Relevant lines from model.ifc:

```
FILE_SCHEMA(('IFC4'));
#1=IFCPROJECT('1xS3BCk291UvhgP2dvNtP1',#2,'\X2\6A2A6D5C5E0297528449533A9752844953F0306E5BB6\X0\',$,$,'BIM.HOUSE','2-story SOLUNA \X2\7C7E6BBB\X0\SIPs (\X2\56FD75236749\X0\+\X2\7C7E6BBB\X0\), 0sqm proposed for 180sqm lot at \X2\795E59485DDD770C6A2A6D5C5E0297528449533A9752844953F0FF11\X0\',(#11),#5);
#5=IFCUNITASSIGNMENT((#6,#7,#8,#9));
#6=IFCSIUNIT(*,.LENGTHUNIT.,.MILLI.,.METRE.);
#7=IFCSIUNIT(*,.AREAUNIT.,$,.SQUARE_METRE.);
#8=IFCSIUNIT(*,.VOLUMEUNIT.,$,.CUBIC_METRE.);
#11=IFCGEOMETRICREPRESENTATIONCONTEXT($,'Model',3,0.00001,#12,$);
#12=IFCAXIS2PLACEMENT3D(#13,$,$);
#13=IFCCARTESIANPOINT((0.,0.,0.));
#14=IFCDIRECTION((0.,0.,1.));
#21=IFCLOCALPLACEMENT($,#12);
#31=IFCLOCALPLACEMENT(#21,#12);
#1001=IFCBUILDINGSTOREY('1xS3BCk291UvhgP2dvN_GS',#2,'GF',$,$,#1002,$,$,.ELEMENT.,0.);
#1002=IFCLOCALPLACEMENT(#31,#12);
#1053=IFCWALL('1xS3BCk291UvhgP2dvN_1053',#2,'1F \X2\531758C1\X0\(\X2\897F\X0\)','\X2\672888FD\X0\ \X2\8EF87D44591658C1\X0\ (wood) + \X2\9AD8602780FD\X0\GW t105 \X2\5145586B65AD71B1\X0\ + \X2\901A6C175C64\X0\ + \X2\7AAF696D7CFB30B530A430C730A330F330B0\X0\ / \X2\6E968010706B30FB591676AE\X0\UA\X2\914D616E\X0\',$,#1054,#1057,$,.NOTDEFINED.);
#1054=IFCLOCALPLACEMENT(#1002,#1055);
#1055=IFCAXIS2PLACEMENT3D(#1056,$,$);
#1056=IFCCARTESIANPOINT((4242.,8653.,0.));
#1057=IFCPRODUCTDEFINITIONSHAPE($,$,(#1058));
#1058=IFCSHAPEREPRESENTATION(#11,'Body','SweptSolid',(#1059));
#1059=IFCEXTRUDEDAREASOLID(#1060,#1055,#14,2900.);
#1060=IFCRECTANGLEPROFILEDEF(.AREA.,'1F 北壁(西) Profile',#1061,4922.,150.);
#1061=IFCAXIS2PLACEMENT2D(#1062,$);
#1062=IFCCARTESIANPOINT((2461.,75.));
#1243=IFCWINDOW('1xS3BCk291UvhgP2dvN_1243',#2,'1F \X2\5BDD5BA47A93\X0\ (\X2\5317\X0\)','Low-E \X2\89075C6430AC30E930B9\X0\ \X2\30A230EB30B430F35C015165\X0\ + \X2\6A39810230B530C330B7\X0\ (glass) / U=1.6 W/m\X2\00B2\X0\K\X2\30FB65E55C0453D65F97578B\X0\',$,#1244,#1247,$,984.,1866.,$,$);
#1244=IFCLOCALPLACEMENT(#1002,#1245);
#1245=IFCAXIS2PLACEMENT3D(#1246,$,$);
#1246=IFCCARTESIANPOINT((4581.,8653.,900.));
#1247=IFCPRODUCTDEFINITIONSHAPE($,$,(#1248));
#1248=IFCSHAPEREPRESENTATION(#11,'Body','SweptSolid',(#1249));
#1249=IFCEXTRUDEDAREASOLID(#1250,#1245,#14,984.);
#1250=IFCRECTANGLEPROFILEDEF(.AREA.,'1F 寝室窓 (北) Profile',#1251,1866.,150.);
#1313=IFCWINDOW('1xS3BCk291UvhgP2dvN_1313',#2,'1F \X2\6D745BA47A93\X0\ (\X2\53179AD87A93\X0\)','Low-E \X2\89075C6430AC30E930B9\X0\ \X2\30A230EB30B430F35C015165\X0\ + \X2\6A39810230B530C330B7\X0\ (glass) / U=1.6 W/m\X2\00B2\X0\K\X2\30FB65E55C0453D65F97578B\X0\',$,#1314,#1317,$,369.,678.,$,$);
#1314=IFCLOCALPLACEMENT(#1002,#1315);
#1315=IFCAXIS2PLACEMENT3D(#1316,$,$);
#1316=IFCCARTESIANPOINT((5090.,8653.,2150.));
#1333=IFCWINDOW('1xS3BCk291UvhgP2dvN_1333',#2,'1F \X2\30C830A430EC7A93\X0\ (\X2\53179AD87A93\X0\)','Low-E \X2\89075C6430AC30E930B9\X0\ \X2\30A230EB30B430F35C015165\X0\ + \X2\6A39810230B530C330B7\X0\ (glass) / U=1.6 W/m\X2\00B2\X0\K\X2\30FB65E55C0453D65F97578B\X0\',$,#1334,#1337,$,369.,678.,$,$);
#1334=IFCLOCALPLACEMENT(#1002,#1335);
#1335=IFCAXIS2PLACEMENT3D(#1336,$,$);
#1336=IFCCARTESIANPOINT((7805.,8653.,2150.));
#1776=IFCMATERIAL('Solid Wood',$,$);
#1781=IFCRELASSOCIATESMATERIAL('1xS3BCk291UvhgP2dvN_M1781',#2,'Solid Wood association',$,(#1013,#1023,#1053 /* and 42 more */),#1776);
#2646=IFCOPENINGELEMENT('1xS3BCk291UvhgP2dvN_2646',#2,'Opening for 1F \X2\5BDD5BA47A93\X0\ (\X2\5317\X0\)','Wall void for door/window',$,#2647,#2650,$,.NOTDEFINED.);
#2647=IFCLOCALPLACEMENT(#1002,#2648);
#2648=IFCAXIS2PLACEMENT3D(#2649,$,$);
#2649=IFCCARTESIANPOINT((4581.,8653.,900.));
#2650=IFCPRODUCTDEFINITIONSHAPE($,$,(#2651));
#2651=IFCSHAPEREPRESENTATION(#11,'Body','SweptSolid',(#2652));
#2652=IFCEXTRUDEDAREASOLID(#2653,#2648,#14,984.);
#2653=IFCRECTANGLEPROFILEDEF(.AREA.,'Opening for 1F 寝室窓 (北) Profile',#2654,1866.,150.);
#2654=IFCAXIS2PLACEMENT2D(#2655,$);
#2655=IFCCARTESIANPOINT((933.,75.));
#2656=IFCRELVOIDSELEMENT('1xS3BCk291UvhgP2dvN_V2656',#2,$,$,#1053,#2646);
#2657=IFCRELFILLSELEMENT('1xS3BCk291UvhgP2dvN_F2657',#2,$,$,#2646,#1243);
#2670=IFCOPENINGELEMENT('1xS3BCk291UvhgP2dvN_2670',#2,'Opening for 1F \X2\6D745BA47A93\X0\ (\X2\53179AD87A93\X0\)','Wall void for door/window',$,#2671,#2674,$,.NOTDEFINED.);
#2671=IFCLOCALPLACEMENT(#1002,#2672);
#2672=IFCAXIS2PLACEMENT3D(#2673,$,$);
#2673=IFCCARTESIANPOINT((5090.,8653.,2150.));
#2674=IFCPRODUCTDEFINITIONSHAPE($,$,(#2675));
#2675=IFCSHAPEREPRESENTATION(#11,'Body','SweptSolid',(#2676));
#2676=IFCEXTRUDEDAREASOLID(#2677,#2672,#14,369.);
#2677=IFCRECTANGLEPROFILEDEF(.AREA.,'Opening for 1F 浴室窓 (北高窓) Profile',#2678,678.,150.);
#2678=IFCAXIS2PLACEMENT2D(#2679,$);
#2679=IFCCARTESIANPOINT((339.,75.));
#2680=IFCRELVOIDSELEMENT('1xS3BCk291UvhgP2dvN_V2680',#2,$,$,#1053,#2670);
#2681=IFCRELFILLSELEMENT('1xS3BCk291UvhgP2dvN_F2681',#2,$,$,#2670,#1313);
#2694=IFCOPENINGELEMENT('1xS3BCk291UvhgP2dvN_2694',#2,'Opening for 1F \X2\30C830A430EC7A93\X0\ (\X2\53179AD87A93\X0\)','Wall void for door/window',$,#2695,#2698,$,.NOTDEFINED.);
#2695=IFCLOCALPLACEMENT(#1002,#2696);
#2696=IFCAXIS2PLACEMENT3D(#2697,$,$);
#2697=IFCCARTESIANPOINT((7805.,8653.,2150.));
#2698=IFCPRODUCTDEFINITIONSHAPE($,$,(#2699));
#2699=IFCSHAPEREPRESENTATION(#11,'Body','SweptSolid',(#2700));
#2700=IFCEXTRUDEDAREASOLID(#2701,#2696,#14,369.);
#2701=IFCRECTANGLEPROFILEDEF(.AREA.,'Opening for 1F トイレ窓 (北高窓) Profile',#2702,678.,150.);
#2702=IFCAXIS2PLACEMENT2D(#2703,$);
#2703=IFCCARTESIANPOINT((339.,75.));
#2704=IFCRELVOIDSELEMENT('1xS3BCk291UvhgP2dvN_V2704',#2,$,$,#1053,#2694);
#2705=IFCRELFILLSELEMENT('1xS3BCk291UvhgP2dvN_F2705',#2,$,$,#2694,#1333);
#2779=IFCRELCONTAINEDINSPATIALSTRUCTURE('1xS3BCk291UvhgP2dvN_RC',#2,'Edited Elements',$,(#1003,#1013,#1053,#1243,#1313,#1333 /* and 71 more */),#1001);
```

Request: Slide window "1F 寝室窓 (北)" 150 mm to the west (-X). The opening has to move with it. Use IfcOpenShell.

```python
import ifcopenshell
import ifcopenshell.api.geometry
import ifcopenshell.util.placement
import ifcopenshell.util.unit

model = ifcopenshell.open("model.ifc")
unit_scale = ifcopenshell.util.unit.calculate_unit_scale(model)

window = model.by_guid("1xS3BCk291UvhgP2dvN_1243")
opening = window.FillsVoids[0].RelatingOpeningElement
wall = opening.VoidsElements[0].RelatingBuildingElement

wall_matrix = ifcopenshell.util.placement.get_local_placement(wall.ObjectPlacement)
shift = wall_matrix[:3, 0] * -0.15 / unit_scale
before = ifcopenshell.util.placement.get_local_placement(window.ObjectPlacement)[:3, 3].copy()

# The window is not placed relative to its opening, so move both.
for product in (opening, window):
    matrix = ifcopenshell.util.placement.get_local_placement(product.ObjectPlacement)
    matrix[:3, 3] += shift
    ifcopenshell.api.geometry.edit_object_placement(model, product=product, matrix=matrix, is_si=False)

after = ifcopenshell.util.placement.get_local_placement(window.ObjectPlacement)[:3, 3]
print("window moved by", (after - before).round(3) + 0.0)

model.write("model_rev.ifc")
```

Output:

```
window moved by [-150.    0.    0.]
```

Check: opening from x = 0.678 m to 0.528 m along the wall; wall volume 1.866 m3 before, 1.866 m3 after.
